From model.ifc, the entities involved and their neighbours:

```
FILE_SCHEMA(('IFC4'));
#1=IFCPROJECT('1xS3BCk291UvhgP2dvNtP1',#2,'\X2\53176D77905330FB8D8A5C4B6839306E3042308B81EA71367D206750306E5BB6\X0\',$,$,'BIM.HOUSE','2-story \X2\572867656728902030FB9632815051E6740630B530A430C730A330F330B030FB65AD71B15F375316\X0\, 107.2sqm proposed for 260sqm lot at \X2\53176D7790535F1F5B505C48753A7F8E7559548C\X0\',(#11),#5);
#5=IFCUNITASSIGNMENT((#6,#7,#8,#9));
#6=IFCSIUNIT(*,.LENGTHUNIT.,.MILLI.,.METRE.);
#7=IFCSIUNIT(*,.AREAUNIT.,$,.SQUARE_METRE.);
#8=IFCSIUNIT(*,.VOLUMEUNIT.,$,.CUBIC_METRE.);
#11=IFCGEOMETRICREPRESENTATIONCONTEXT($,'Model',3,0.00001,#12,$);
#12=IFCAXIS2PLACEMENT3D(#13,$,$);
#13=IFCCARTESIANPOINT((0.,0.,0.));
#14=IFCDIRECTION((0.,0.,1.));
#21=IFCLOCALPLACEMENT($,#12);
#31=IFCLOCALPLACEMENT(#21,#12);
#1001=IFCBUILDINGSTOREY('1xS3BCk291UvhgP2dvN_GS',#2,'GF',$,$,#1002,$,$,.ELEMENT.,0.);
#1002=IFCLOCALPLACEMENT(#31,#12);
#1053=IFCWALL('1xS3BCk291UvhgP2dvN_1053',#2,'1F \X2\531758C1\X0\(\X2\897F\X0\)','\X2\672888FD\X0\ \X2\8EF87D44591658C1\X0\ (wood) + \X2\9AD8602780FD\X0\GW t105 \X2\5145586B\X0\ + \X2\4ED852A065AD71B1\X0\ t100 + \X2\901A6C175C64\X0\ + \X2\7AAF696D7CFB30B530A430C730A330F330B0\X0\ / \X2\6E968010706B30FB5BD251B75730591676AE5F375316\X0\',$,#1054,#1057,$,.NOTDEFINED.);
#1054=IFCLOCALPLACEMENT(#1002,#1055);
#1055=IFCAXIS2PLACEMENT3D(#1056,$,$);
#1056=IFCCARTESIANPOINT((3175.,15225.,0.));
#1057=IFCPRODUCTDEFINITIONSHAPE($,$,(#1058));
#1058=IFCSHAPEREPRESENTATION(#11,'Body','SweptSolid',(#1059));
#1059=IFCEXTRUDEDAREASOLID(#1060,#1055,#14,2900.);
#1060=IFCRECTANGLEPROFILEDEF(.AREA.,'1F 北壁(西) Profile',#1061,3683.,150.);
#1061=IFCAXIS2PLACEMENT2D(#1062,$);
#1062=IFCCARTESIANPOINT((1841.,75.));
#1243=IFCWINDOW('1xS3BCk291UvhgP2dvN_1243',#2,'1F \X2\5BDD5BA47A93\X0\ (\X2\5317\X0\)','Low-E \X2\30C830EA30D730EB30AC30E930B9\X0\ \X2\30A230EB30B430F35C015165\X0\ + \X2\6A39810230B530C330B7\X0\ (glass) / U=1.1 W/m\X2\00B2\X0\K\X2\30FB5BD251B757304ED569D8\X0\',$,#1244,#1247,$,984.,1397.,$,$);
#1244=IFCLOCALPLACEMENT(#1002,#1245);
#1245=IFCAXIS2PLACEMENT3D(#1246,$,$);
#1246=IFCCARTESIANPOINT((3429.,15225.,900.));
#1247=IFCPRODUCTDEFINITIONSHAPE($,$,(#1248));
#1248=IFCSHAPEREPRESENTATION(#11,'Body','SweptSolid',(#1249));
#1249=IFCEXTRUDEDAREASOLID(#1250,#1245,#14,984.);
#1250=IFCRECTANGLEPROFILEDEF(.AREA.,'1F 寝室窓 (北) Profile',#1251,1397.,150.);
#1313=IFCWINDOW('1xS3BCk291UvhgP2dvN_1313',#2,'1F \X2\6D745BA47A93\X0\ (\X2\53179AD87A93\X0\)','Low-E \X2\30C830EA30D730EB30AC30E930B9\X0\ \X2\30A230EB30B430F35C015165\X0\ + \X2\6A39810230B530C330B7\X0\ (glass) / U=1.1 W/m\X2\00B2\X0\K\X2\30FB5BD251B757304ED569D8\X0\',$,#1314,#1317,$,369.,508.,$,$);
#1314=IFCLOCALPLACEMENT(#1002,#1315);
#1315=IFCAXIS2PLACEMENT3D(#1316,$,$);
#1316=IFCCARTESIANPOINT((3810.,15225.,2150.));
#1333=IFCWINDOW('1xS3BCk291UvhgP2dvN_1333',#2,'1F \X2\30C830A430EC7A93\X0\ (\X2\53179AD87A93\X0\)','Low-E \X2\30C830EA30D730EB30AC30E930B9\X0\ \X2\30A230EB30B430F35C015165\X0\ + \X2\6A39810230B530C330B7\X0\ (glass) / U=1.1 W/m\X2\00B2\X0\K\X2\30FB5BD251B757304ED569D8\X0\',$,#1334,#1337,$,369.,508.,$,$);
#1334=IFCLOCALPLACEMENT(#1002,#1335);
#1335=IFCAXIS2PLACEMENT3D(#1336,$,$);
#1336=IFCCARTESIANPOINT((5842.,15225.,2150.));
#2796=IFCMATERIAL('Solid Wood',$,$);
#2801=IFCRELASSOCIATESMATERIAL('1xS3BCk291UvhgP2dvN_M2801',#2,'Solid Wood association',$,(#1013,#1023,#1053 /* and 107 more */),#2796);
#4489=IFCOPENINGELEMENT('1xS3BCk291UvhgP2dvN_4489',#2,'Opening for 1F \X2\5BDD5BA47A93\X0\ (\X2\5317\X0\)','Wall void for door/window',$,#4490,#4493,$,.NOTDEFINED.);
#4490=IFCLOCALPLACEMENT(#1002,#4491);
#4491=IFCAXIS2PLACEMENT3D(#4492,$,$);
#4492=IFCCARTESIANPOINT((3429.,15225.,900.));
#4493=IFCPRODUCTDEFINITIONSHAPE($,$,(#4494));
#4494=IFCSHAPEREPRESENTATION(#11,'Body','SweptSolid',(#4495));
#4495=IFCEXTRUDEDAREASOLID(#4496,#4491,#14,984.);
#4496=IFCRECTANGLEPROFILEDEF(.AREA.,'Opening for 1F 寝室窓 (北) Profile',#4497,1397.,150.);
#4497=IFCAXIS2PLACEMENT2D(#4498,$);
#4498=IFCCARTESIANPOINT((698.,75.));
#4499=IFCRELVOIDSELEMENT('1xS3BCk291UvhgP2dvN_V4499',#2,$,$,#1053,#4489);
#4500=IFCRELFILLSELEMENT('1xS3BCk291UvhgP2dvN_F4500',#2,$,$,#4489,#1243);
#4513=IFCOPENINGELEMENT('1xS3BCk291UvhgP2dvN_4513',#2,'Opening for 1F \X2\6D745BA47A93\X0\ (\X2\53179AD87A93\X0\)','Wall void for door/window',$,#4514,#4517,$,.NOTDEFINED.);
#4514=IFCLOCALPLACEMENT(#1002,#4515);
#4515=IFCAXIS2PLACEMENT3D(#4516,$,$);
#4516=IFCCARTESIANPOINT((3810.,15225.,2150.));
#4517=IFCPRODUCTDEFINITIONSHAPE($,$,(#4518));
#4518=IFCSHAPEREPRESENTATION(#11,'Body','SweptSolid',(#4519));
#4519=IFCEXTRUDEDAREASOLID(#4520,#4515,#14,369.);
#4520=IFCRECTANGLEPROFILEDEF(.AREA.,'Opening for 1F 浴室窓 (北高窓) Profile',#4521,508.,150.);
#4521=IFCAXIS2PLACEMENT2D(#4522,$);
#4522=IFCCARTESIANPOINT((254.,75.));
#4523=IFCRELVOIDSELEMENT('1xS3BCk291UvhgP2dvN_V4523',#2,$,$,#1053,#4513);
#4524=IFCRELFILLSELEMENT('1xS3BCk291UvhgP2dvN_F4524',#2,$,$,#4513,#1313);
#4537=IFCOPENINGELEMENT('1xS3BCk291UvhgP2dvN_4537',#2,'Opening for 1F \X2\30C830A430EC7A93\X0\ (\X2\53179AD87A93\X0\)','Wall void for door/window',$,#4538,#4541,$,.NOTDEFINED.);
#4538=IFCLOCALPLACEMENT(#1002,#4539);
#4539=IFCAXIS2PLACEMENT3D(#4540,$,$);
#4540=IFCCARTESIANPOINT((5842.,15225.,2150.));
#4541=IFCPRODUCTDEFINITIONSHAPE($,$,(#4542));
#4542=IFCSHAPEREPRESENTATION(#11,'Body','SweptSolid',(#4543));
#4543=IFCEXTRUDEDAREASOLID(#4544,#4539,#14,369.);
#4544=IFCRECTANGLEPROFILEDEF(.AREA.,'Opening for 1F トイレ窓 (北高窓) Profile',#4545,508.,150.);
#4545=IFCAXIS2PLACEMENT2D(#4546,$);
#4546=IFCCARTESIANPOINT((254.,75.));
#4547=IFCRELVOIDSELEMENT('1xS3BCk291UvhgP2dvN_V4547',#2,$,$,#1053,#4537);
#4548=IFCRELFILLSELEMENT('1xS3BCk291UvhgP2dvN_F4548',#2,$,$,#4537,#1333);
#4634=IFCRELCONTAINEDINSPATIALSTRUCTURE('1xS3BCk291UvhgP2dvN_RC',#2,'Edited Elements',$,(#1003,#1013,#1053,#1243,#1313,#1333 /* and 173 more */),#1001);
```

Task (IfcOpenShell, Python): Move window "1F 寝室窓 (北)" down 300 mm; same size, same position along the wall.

```python
import numpy as np
import ifcopenshell
import ifcopenshell.api.geometry
import ifcopenshell.util.placement
import ifcopenshell.util.unit

model = ifcopenshell.open("model.ifc")
unit_scale = ifcopenshell.util.unit.calculate_unit_scale(model)

window = model.by_guid("1xS3BCk291UvhgP2dvN_1243")
opening = window.FillsVoids[0].RelatingOpeningElement
dz = -300.0

shift = np.array([0.0, 0.0, dz])
# The window is not placed relative to its opening, so move both.
for product in (opening, window):
    matrix = ifcopenshell.util.placement.get_local_placement(product.ObjectPlacement)
    matrix[:3, 3] += shift
    ifcopenshell.api.geometry.edit_object_placement(model, product=product, matrix=matrix, is_si=False)

print(f"moved by {dz * unit_scale:+.3f} m")

model.write("model_updated.ifc")
```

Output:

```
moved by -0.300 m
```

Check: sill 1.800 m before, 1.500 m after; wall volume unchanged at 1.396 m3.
